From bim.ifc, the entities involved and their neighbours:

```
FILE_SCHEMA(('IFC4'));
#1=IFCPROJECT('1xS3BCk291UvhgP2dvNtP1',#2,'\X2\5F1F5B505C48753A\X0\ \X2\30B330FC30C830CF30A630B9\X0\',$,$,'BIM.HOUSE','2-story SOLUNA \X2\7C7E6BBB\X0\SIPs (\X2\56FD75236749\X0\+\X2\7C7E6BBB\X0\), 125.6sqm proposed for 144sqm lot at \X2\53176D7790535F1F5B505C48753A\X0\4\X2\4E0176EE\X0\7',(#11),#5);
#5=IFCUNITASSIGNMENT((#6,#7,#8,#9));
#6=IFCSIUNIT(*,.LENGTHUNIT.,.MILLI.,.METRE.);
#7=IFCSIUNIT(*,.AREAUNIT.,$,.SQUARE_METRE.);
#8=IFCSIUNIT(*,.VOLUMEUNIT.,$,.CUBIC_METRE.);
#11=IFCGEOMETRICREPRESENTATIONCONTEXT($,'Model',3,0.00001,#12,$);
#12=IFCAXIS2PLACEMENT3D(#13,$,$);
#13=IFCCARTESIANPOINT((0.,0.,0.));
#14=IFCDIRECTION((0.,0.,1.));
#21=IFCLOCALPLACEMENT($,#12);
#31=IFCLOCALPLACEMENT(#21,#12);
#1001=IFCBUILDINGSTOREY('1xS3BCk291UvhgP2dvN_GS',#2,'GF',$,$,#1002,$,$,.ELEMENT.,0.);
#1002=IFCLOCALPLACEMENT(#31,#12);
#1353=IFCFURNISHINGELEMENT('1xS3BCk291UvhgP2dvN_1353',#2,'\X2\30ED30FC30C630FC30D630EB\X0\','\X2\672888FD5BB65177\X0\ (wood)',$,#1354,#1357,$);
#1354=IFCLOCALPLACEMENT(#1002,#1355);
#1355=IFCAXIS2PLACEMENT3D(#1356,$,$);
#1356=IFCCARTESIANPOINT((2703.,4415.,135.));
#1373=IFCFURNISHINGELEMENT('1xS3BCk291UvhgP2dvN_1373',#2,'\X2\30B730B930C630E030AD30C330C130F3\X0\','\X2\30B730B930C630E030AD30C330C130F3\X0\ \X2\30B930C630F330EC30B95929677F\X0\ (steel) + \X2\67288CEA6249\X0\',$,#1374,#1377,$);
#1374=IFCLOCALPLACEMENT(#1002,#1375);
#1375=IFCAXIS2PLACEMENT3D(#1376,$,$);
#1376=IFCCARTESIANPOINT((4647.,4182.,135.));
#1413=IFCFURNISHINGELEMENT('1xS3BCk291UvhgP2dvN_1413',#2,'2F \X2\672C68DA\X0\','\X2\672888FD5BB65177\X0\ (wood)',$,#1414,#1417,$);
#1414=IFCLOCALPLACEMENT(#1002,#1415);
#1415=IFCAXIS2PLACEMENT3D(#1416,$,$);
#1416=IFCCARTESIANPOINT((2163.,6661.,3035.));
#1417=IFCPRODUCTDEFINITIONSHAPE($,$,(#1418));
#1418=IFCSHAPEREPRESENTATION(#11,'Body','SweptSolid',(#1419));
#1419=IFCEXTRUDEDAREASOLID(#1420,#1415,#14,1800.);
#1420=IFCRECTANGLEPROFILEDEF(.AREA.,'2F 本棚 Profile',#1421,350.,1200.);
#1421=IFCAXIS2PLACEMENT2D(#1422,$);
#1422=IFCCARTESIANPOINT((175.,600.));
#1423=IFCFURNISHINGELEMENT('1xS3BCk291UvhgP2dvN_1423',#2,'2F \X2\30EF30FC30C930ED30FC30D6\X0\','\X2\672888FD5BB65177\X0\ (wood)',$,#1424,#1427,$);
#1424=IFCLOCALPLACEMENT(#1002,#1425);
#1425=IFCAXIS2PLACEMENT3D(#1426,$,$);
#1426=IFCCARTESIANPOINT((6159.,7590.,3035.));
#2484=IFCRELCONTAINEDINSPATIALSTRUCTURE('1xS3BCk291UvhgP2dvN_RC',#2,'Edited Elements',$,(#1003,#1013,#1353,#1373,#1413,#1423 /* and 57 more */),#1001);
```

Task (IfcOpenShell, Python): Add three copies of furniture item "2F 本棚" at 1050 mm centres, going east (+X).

```python
import numpy as np
import ifcopenshell
import ifcopenshell.api.geometry
import ifcopenshell.api.root
import ifcopenshell.util.element
import ifcopenshell.util.placement

model = ifcopenshell.open("bim.ifc")


def reuse_history(source, copy):
    """copy_class also copies each property set's owner history, people and application; keep the originals."""
    for rel in copy.IsDefinedBy:
        if rel.is_a("IfcRelDefinesByProperties") and (history := rel.RelatingPropertyDefinition.OwnerHistory):
            rel.RelatingPropertyDefinition.OwnerHistory = source.OwnerHistory
            ifcopenshell.util.element.remove_deep2(model, history)


source = model.by_guid("1xS3BCk291UvhgP2dvN_1413")
base = ifcopenshell.util.placement.get_local_placement(source.ObjectPlacement)
step = np.array([1.0, 0.0, 0.0]) * 1050.0

for i in range(1, 4):
    copy = ifcopenshell.api.root.copy_class(model, product=source)
    copy.Representation = ifcopenshell.util.element.copy_deep(
        model, source.Representation, exclude=["IfcGeometricRepresentationContext", "IfcRepresentationMap"]
    )
    reuse_history(source, copy)
    matrix = base.copy()
    matrix[:3, 3] += i * step
    print("added at", matrix[:3, 3].round(3) + 0.0)
    ifcopenshell.api.geometry.edit_object_placement(model, product=copy, matrix=matrix, is_si=False)

model.write("bim_v2.ifc")
```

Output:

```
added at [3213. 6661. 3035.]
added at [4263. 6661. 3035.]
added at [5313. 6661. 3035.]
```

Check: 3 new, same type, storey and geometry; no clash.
